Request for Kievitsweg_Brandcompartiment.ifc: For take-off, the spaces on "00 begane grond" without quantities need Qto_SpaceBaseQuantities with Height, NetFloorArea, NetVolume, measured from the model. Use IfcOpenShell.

First a look at what the model holds.

```python
import ifcopenshell
import ifcopenshell.util.element
import ifcopenshell.util.unit

model = ifcopenshell.open("Kievitsweg_Brandcompartiment.ifc")
print(model.schema)
for unit_type in ("LENGTHUNIT", "AREAUNIT", "VOLUMEUNIT"):
    print(unit_type, ifcopenshell.util.unit.calculate_unit_scale(model, unit_type))
storey = next(s for s in model.by_type("IfcBuildingStorey") if s.Name == "00 begane grond")
spaces = [e for e in ifcopenshell.util.element.get_decomposition(storey) if e.is_a("IfcSpace")]
for e in sorted(spaces, key=lambda e: e.id()):
    print(e.id(), e.is_a(), e.Name, list(ifcopenshell.util.element.get_psets(e, qtos_only=True)), sep=" | ")
```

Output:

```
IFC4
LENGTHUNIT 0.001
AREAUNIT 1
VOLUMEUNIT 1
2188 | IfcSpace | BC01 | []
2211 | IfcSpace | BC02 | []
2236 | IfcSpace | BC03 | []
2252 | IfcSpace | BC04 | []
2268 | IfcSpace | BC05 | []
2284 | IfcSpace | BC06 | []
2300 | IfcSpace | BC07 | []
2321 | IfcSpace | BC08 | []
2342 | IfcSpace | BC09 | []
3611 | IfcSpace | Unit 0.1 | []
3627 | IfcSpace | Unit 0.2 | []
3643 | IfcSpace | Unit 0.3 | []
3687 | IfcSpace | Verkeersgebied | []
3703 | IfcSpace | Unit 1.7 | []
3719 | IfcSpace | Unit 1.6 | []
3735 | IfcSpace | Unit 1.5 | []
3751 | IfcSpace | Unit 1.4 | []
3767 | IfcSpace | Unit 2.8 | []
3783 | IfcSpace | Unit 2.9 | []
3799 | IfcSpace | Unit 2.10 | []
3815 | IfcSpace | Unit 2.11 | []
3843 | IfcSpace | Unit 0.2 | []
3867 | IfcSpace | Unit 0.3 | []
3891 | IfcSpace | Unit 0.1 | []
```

```python
import ifcopenshell
import ifcopenshell.api.pset
import ifcopenshell.geom
import ifcopenshell.util.element
import ifcopenshell.util.shape
import ifcopenshell.util.unit

model = ifcopenshell.open("Kievitsweg_Brandcompartiment.ifc")
unit_scale = ifcopenshell.util.unit.calculate_unit_scale(model)
area_scale = ifcopenshell.util.unit.calculate_unit_scale(model, "AREAUNIT")
volume_scale = ifcopenshell.util.unit.calculate_unit_scale(model, "VOLUMEUNIT")
settings = ifcopenshell.geom.settings()

storey = next(s for s in model.by_type("IfcBuildingStorey") if s.Name == "00 begane grond")
spaces = [e for e in ifcopenshell.util.element.get_decomposition(storey) if e.is_a("IfcSpace")]

for e in sorted(spaces, key=lambda e: e.id()):
    if ifcopenshell.util.element.get_psets(e, qtos_only=True, should_inherit=False):
        continue
    # Geometry comes back in metres, in the element's own axes.
    shape = ifcopenshell.geom.create_shape(settings, e)
    values = {
        "Height": ifcopenshell.util.shape.get_z(shape.geometry) / unit_scale,
        "NetFloorArea": ifcopenshell.util.shape.get_footprint_area(shape.geometry) / area_scale,
        "NetVolume": ifcopenshell.util.shape.get_volume(shape.geometry) / volume_scale,
    }
    qto = ifcopenshell.api.pset.add_qto(model, product=e, name="Qto_SpaceBaseQuantities")
    ifcopenshell.api.pset.edit_qto(model, qto=qto, properties=values)
    print(e.id(), {k: round(v, 3) for k, v in values.items()})

model.write("Kievitsweg_Brandcompartiment_edited.ifc")
```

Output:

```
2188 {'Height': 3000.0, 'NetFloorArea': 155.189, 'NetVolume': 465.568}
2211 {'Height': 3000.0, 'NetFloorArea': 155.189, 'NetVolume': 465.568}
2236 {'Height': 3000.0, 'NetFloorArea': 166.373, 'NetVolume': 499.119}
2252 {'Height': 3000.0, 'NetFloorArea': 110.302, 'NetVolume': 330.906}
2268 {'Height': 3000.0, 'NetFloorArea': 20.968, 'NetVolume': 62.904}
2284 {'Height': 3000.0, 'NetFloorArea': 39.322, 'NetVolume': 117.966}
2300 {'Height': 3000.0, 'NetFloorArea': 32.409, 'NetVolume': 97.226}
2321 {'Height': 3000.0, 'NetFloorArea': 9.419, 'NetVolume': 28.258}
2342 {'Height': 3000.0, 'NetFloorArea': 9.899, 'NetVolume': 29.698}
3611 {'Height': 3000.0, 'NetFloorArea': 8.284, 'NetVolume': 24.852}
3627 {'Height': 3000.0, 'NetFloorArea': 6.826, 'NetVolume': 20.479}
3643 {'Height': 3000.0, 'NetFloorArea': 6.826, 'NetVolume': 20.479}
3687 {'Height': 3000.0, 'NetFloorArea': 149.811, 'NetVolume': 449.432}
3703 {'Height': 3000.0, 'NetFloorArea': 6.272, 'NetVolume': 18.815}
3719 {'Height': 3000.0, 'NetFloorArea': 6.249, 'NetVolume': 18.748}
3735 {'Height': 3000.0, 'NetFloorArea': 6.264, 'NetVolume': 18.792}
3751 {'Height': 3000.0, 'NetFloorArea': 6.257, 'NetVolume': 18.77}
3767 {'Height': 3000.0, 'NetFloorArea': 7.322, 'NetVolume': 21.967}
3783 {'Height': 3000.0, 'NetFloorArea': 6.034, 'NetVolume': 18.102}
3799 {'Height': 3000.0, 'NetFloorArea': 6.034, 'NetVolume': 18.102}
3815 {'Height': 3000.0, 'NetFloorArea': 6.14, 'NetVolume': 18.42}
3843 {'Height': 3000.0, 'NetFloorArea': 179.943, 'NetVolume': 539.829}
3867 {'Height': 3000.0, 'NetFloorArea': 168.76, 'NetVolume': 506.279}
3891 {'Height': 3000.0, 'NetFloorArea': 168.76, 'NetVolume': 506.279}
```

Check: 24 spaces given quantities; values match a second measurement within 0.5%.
